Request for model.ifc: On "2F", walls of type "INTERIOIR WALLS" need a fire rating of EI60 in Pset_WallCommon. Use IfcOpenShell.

First a look at what the model holds.

```python
import ifcopenshell
import ifcopenshell.util.element

model = ifcopenshell.open("model.ifc")
print(model.schema)
storey = next(s for s in model.by_type("IfcBuildingStorey") if s.Name == "2F")
walls = [e for e in ifcopenshell.util.element.get_decomposition(storey) if e.is_a("IfcWall")]
seen = {}
for e in walls:
    element_type = ifcopenshell.util.element.get_type(e)
    key = (element_type.Name if element_type != e and element_type else None, ifcopenshell.util.element.get_pset(e, "Pset_WallCommon", "FireRating"))
    seen[key] = seen.get(key, 0) + 1
for (name, value), count in sorted(seen.items(), key=str):
    print(count, "x", name, "|", value)
```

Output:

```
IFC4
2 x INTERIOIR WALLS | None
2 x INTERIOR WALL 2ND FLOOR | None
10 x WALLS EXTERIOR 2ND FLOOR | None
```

```python
import ifcopenshell
import ifcopenshell.api.pset
import ifcopenshell.util.element

model = ifcopenshell.open("model.ifc")

storey = next(s for s in model.by_type("IfcBuildingStorey") if s.Name == "2F")
walls = [e for e in ifcopenshell.util.element.get_decomposition(storey) if e.is_a("IfcWall")]

count = 0
for e in walls:
    element_type = ifcopenshell.util.element.get_type(e)
    if element_type in (None, e) or element_type.Name != "INTERIOIR WALLS":
        continue
    # add_pset returns the element's existing set when there is one.
    pset = ifcopenshell.api.pset.add_pset(model, product=e, name="Pset_WallCommon")
    ifcopenshell.api.pset.edit_pset(model, pset=pset, properties={"FireRating": "EI60"})
    count += 1

print(count, "walls updated")

model.write("model_rev.ifc")
```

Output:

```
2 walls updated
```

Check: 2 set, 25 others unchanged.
